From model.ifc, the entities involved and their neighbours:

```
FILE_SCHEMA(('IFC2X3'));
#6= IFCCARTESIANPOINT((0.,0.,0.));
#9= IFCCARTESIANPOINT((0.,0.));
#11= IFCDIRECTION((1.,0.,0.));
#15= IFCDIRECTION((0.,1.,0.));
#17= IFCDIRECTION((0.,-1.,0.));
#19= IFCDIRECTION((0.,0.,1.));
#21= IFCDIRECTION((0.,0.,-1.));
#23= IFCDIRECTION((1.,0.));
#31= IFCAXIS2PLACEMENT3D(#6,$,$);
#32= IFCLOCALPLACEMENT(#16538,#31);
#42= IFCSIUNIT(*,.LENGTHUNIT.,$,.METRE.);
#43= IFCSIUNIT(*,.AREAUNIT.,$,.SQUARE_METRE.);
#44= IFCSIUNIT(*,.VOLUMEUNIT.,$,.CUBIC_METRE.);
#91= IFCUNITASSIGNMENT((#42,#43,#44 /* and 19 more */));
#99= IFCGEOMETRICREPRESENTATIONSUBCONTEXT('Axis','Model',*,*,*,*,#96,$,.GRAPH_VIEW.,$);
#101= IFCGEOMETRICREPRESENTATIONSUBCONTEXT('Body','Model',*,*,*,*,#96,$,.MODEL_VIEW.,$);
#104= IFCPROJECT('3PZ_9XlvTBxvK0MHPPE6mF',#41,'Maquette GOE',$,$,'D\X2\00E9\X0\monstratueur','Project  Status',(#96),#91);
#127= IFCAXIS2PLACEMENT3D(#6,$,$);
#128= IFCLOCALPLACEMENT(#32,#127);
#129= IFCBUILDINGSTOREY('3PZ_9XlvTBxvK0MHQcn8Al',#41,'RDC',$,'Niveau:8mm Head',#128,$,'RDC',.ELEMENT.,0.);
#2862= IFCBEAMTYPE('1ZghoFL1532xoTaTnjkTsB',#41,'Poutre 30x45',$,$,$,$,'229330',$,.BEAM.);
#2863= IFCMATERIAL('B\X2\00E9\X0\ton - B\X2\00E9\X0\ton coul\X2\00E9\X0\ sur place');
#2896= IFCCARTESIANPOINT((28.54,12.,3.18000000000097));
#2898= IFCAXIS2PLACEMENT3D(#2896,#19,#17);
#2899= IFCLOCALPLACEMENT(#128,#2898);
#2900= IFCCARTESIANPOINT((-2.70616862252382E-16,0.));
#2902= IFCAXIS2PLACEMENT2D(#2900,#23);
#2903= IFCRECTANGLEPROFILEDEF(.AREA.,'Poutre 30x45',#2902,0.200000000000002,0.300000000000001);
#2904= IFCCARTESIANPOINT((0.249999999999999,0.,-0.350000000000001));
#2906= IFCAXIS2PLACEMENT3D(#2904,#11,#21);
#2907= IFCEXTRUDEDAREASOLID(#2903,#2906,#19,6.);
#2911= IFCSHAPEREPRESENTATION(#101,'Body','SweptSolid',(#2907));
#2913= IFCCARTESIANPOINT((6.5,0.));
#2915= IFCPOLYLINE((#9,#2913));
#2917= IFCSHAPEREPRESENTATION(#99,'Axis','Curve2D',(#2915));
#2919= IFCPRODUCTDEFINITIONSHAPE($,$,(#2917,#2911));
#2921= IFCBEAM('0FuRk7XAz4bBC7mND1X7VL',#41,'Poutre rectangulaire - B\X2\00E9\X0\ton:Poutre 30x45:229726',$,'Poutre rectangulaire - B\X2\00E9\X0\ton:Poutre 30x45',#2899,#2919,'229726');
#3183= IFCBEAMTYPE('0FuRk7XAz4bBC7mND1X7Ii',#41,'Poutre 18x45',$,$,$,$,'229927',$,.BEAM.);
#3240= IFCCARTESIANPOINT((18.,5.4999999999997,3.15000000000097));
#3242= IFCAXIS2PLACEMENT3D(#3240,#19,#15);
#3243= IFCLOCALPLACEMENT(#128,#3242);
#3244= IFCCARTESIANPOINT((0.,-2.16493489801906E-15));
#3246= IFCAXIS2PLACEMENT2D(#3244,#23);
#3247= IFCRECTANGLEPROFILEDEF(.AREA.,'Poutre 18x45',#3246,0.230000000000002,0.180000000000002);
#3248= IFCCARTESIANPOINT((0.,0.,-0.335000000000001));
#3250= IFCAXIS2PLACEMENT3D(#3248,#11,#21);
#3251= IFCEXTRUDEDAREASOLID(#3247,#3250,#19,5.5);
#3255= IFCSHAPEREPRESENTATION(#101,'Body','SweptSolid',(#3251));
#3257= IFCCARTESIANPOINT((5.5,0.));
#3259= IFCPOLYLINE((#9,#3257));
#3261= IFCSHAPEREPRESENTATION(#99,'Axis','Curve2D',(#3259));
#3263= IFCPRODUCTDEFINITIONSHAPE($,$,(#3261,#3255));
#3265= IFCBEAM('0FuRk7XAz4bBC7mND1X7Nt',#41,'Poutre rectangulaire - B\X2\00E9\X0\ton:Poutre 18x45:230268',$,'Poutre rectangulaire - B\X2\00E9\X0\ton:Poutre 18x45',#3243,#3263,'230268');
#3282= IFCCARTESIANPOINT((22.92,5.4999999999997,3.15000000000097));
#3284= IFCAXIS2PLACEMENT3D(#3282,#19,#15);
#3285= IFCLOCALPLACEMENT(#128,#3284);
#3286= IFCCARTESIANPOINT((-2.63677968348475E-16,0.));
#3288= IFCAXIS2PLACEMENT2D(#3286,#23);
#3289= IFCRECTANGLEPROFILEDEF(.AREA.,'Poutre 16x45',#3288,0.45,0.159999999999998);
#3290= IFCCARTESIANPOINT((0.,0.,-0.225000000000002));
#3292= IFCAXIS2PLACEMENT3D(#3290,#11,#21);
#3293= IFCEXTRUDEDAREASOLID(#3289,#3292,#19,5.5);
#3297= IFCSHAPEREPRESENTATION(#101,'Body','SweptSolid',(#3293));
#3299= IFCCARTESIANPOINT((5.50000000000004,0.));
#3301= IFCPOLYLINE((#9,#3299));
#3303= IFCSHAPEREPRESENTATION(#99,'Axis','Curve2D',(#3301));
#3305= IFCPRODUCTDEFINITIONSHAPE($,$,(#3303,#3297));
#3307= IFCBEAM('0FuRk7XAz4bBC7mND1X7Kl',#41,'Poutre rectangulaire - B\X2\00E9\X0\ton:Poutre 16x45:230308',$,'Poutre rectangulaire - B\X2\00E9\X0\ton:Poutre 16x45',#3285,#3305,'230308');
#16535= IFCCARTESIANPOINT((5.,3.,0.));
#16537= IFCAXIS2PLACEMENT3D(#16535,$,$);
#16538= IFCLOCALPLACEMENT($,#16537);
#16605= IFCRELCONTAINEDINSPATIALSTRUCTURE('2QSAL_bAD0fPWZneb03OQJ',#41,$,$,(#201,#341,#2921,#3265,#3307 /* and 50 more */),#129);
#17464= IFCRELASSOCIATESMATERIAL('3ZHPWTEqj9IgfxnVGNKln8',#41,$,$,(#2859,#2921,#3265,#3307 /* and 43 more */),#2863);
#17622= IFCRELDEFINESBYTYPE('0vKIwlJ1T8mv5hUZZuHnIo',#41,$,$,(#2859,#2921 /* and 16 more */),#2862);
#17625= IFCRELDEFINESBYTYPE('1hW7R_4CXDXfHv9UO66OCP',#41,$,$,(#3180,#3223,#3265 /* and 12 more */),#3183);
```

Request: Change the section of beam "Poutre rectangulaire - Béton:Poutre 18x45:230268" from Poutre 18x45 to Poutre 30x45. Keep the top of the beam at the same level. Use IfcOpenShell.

```python
import ifcopenshell
import ifcopenshell.api.type
import ifcopenshell.util.element
import ifcopenshell.util.representation

model = ifcopenshell.open("model.ifc")

member = model.by_guid("0FuRk7XAz4bBC7mND1X7Nt")
source = next(p for p in model.by_type("IfcRectangleProfileDef") if p.ProfileName == "Poutre 30x45")

body = ifcopenshell.util.representation.get_representation(member, "Model", "Body")
solid = body.Items[0]
old_profile = solid.SweptArea

# Copy the section's sizes but keep this member's own profile position.
profile = ifcopenshell.util.element.copy(model, source)
# Profiles are centred, so shift by half the change in depth to hold the top.
shift = (old_profile.XDim - profile.XDim) / 2
x, y = old_profile.Position.Location.Coordinates
up = (-1.0, 0.0)  # upwards, in the solid's own plane
location = model.createIfcCartesianPoint((x + up[0] * shift, y + up[1] * shift))
profile.Position = model.createIfcAxis2Placement2D(location, old_profile.Position.RefDirection)
solid.SweptArea = profile
if not model.get_total_inverses(old_profile):
    ifcopenshell.util.element.remove_deep2(model, old_profile)

new_type = model.by_id(2862)
ifcopenshell.api.type.assign_type(
    model, related_objects=[member], relating_type=new_type, should_map_representations=False
)
member.Name = member.Name.replace("Poutre 18x45", "Poutre 30x45")
member.ObjectType = "Poutre rectangulaire - Béton:Poutre 30x45"

print(solid.SweptArea)

model.write("model_v2.ifc")
```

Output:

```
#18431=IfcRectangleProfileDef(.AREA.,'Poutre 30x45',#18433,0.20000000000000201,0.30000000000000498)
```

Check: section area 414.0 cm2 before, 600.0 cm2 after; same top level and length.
